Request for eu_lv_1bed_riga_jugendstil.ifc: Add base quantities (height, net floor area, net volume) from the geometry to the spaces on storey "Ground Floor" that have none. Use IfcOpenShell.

First a look at what the model holds.

```python
import ifcopenshell
import ifcopenshell.util.element
import ifcopenshell.util.unit

model = ifcopenshell.open("eu_lv_1bed_riga_jugendstil.ifc")
print(model.schema)
for unit_type in ("LENGTHUNIT", "AREAUNIT", "VOLUMEUNIT"):
    print(unit_type, ifcopenshell.util.unit.calculate_unit_scale(model, unit_type))
storey = next(s for s in model.by_type("IfcBuildingStorey") if s.Name == "Ground Floor")
spaces = [e for e in ifcopenshell.util.element.get_decomposition(storey) if e.is_a("IfcSpace")]
for e in sorted(spaces, key=lambda e: e.id()):
    print(e.id(), e.is_a(), e.Name, list(ifcopenshell.util.element.get_psets(e, qtos_only=True)), sep=" | ")
```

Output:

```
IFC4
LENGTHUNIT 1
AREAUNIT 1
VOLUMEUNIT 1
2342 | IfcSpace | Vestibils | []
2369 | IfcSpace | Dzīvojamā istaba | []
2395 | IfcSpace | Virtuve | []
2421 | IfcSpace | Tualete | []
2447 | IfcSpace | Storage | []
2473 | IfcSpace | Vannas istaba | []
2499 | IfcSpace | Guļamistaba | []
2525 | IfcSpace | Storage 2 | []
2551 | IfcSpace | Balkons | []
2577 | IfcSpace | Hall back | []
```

```python
import ifcopenshell
import ifcopenshell.api.pset
import ifcopenshell.geom
import ifcopenshell.util.element
import ifcopenshell.util.shape
import ifcopenshell.util.unit

model = ifcopenshell.open("eu_lv_1bed_riga_jugendstil.ifc")
unit_scale = ifcopenshell.util.unit.calculate_unit_scale(model)
area_scale = ifcopenshell.util.unit.calculate_unit_scale(model, "AREAUNIT")
volume_scale = ifcopenshell.util.unit.calculate_unit_scale(model, "VOLUMEUNIT")
settings = ifcopenshell.geom.settings()

storey = next(s for s in model.by_type("IfcBuildingStorey") if s.Name == "Ground Floor")
spaces = [e for e in ifcopenshell.util.element.get_decomposition(storey) if e.is_a("IfcSpace")]

for e in sorted(spaces, key=lambda e: e.id()):
    if ifcopenshell.util.element.get_psets(e, qtos_only=True, should_inherit=False):
        continue
    # Geometry comes back in metres, in the element's own axes.
    shape = ifcopenshell.geom.create_shape(settings, e)
    values = {
        "Height": ifcopenshell.util.shape.get_z(shape.geometry) / unit_scale,
        "NetFloorArea": ifcopenshell.util.shape.get_footprint_area(shape.geometry) / area_scale,
        "NetVolume": ifcopenshell.util.shape.get_volume(shape.geometry) / volume_scale,
    }
    qto = ifcopenshell.api.pset.add_qto(model, product=e, name="Qto_SpaceBaseQuantities")
    ifcopenshell.api.pset.edit_qto(model, qto=qto, properties=values)
    print(e.id(), {k: round(v, 3) for k, v in values.items()})

model.write("eu_lv_1bed_riga_jugendstil-out.ifc")
```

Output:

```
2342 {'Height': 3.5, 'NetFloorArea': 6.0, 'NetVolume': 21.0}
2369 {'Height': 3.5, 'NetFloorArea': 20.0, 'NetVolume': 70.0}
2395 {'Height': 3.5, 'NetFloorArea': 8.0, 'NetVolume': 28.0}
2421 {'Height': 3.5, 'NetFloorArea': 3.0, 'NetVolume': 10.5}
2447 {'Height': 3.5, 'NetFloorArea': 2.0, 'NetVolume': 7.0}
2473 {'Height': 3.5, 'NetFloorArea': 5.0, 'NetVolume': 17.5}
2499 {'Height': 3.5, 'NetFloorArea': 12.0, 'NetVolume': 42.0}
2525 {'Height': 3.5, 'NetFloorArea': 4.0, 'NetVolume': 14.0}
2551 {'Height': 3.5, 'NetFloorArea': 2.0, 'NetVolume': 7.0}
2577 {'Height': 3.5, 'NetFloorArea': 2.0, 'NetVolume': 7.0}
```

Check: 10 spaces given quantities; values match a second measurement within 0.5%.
